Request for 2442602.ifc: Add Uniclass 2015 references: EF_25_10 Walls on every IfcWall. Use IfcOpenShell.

First a look at what the model holds.

```python
import ifcopenshell

model = ifcopenshell.open("2442602.ifc")
print(model.schema)
print("classifications:", [c.Name for c in model.by_type("IfcClassification")])
for ifc_class in ("IfcDoor", "IfcRoof", "IfcStair", "IfcWall", "IfcWindow"):
    print(ifc_class, len(model.by_type(ifc_class)))
```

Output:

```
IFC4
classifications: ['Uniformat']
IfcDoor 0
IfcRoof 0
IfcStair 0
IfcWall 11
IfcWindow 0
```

```python
import ifcopenshell
import ifcopenshell.api.classification

model = ifcopenshell.open("2442602.ifc")

system = ifcopenshell.api.classification.add_classification(model, classification="Uniclass 2015")

codes = {
    "IfcWall": ("EF_25_10", "Walls"),
}
for ifc_class, (code, name) in codes.items():
    products = model.by_type(ifc_class)
    ifcopenshell.api.classification.add_reference(
        model, products=products, classification=system, identification=code, name=name
    )
    print(code, len(products))

model.write("2442602_rev.ifc")
```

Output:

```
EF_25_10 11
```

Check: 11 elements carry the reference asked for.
